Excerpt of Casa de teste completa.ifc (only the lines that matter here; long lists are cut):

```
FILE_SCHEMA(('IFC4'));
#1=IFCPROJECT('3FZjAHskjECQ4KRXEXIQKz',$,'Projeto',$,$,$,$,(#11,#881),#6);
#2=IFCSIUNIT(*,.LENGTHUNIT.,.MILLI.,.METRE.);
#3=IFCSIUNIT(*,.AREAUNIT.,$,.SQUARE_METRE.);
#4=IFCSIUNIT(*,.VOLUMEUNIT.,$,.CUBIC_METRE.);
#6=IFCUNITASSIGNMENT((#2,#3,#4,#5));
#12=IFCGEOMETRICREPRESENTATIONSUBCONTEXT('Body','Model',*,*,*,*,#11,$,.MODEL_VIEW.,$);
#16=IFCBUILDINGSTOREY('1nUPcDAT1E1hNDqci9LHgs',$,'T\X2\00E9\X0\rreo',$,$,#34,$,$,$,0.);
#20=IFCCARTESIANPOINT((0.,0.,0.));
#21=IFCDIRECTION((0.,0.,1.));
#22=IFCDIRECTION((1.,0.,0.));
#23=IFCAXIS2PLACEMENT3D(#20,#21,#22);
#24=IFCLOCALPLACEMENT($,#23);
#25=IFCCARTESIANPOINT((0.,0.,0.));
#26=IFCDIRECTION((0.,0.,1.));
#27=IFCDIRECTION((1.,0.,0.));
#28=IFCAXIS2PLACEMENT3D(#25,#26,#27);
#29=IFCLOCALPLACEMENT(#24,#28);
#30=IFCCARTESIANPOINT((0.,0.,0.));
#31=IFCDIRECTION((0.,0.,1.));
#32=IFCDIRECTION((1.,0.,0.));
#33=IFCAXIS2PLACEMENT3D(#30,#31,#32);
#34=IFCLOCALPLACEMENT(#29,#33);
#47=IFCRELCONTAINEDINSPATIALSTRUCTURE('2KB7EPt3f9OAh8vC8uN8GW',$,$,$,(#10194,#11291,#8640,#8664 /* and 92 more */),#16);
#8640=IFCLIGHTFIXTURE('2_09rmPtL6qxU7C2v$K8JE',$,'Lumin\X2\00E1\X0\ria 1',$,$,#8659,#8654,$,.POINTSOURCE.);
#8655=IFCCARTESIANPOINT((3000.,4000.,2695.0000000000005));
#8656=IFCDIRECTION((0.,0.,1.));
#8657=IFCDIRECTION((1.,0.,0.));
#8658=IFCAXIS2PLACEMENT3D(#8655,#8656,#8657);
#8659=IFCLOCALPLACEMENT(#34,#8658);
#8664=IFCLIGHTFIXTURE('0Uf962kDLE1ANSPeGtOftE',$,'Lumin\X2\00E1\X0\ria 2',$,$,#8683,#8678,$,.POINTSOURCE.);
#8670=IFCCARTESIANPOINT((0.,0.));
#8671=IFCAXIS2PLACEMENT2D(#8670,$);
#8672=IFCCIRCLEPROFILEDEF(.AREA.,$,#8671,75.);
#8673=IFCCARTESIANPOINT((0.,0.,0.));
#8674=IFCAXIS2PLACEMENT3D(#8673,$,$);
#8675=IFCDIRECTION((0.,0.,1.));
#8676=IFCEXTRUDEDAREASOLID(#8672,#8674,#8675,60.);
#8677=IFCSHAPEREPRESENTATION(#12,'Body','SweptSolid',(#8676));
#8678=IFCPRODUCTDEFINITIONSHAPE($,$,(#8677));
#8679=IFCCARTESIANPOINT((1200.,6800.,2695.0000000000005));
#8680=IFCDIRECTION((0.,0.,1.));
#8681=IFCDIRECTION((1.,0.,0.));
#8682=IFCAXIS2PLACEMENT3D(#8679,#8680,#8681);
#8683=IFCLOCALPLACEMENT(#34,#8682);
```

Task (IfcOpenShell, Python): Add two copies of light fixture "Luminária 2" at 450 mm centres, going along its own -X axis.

```python
import ifcopenshell
import ifcopenshell.api.geometry
import ifcopenshell.api.root
import ifcopenshell.util.element
import ifcopenshell.util.placement

model = ifcopenshell.open("Casa de teste completa.ifc")

source = model.by_guid("0Uf962kDLE1ANSPeGtOftE")
base = ifcopenshell.util.placement.get_local_placement(source.ObjectPlacement)
step = -base[:3, 0] * 450.0

for i in range(1, 3):
    copy = ifcopenshell.api.root.copy_class(model, product=source)
    copy.Representation = ifcopenshell.util.element.copy_deep(
        model, source.Representation, exclude=["IfcGeometricRepresentationContext", "IfcRepresentationMap"]
    )
    matrix = base.copy()
    matrix[:3, 3] += i * step
    print("added at", matrix[:3, 3].round(3) + 0.0)
    ifcopenshell.api.geometry.edit_object_placement(model, product=copy, matrix=matrix, is_si=False)

model.write("Casa de teste completa_rev.ifc")
```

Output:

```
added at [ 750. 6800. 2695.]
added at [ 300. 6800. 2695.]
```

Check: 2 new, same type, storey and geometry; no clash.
